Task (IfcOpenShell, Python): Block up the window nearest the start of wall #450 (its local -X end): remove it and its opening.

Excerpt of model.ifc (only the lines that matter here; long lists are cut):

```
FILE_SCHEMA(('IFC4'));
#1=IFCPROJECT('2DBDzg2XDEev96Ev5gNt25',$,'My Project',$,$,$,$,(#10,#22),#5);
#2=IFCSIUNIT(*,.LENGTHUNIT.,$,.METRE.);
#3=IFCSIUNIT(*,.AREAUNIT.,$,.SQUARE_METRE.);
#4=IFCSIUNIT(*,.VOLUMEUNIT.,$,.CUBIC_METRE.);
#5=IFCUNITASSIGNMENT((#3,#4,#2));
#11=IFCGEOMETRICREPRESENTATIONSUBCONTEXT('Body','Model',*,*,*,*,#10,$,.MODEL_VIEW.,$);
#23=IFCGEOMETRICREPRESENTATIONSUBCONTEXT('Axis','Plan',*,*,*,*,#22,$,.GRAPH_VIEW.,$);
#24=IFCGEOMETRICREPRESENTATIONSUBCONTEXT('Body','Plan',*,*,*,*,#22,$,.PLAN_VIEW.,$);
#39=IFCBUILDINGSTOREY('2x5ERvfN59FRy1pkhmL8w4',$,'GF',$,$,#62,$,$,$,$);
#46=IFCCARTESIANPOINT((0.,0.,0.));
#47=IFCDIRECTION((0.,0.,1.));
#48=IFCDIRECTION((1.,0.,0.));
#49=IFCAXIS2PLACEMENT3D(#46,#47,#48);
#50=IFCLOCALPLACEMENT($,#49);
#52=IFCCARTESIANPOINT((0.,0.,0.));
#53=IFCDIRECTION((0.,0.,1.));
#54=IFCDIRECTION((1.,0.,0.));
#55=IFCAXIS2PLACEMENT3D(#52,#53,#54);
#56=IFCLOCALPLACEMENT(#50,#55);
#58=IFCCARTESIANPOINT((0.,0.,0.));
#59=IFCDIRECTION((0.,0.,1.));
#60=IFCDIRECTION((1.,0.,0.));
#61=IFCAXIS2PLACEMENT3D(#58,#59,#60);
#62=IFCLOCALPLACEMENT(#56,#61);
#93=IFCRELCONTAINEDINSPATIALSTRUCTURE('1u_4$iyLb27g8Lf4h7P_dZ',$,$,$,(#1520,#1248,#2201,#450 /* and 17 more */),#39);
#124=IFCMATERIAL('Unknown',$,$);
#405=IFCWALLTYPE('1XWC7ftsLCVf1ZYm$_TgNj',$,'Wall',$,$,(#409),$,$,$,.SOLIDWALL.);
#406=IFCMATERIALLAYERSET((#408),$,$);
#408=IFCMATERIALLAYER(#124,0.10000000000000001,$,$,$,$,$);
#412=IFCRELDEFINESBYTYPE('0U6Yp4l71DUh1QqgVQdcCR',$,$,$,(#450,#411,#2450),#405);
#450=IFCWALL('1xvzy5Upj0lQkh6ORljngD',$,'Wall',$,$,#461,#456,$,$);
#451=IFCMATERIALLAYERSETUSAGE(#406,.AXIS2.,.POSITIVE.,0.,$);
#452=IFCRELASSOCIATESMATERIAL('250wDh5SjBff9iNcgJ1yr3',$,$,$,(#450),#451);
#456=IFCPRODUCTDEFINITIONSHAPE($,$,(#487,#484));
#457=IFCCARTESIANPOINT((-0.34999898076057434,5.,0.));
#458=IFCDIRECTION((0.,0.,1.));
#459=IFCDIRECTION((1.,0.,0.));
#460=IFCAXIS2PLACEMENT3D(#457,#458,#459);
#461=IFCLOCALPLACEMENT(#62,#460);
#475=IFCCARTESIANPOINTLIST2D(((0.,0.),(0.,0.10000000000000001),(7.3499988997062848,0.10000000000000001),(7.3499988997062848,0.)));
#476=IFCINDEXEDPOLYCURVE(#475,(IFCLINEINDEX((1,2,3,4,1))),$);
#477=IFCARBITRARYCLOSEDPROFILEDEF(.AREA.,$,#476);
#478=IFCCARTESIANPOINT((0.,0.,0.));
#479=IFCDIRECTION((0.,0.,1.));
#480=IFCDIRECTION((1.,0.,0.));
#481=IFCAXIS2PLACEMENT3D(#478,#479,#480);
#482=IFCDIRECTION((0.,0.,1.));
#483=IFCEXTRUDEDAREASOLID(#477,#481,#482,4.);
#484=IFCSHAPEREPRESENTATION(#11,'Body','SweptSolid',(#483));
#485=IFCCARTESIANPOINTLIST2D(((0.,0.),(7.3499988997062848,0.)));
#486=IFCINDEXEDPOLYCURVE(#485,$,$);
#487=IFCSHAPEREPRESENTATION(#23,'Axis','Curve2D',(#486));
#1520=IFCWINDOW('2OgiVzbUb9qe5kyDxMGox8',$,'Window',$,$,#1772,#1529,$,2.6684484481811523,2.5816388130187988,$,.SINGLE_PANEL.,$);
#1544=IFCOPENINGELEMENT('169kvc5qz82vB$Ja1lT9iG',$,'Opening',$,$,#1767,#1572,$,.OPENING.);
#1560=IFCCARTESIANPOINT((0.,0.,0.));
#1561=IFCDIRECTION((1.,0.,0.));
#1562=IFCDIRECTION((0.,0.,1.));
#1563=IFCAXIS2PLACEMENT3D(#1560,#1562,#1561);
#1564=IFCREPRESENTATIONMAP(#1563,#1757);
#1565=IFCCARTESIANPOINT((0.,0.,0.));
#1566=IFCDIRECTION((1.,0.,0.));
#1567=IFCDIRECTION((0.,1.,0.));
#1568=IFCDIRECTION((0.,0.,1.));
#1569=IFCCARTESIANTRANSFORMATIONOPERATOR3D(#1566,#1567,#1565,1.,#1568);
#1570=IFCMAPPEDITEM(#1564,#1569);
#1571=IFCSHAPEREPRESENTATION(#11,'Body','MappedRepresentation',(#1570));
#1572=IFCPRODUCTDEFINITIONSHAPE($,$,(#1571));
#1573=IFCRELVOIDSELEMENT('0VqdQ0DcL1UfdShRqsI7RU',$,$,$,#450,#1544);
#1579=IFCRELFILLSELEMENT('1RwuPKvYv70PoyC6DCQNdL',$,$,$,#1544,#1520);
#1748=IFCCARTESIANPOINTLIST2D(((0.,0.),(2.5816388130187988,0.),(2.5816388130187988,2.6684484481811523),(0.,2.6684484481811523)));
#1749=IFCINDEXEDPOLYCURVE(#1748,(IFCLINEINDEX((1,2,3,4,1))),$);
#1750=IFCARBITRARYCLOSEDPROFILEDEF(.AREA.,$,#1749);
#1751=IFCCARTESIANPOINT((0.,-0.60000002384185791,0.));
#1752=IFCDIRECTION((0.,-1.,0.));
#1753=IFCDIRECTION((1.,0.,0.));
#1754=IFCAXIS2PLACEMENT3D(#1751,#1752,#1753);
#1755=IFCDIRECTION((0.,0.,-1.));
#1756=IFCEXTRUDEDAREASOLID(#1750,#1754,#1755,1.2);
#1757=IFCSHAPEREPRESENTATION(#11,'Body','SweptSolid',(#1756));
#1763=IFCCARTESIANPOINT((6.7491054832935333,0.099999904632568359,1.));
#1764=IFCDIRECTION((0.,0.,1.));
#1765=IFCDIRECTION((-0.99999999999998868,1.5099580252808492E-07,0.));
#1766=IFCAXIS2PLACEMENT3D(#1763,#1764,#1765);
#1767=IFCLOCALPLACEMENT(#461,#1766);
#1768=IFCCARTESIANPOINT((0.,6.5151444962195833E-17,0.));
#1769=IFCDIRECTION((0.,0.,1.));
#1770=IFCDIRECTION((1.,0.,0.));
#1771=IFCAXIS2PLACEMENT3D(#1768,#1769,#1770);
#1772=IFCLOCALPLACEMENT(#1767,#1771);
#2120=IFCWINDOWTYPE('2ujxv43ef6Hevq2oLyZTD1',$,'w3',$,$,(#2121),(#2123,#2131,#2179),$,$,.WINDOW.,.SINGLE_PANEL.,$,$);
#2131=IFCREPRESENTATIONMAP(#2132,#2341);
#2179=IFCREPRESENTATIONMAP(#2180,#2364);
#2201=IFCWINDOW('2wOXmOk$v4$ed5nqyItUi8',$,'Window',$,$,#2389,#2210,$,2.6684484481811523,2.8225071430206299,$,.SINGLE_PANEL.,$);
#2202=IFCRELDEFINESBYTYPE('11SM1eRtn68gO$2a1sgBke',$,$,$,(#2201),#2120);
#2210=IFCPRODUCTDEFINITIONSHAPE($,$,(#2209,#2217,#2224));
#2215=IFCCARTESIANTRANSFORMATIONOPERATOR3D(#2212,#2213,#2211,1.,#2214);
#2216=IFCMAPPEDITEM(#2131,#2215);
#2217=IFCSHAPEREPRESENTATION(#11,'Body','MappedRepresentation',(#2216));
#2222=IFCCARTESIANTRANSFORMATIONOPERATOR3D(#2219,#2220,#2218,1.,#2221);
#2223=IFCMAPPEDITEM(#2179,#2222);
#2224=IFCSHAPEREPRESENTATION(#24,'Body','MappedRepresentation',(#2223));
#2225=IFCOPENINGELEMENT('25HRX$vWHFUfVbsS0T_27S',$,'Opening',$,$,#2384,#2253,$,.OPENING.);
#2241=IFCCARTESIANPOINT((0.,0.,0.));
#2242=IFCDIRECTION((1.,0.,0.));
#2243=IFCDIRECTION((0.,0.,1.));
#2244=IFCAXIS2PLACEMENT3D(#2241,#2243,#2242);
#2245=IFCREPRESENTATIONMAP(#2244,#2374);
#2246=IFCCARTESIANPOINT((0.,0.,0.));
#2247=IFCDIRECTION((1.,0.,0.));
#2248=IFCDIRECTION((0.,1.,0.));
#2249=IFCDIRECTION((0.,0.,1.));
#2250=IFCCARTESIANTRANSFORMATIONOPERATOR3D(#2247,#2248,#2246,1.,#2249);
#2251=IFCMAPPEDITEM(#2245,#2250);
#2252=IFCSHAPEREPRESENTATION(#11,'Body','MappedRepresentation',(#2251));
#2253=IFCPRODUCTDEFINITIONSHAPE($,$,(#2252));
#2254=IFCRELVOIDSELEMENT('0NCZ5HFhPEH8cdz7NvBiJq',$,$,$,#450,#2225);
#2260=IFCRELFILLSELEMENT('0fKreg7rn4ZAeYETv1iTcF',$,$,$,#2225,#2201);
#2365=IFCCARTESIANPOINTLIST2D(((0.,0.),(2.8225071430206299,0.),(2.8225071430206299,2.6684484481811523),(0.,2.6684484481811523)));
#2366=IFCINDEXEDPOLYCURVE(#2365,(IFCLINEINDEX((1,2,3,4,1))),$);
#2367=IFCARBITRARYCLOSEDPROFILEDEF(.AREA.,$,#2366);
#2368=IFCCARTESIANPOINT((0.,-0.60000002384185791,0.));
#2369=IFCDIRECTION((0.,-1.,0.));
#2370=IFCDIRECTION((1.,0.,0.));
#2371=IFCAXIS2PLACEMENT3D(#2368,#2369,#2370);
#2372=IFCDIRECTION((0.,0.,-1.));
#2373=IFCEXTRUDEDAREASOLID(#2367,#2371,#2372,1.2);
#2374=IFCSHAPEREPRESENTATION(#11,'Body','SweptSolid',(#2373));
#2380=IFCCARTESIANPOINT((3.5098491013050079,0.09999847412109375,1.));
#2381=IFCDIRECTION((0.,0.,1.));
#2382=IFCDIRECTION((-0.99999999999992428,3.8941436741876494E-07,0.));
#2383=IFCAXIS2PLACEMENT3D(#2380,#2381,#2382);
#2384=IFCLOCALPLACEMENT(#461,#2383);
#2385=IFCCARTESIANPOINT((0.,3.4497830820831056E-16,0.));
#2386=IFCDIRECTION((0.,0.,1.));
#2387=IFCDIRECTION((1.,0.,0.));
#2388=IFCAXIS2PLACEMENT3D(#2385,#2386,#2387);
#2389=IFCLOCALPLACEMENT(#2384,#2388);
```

```python
import ifcopenshell
import ifcopenshell.api.feature
import ifcopenshell.api.root
import ifcopenshell.geom
import ifcopenshell.util.shape

model = ifcopenshell.open("model.ifc")
settings = ifcopenshell.geom.settings()


def volume(element):
    """Net volume in cubic metres, openings subtracted."""
    shape = ifcopenshell.geom.create_shape(settings, element)
    return ifcopenshell.util.shape.get_volume(shape.geometry)


window = model.by_id(2201)
opening = window.FillsVoids[0].RelatingOpeningElement
wall = opening.VoidsElements[0].RelatingBuildingElement
before = volume(wall)

ifcopenshell.api.root.remove_product(model, product=window)
ifcopenshell.api.feature.remove_feature(model, feature=opening)

after = volume(wall)

print(f"wall volume {before:.3f} -> {after:.3f} m3")

model.write("model_v2.ifc")
```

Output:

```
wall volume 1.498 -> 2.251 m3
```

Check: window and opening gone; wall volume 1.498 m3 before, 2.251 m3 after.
